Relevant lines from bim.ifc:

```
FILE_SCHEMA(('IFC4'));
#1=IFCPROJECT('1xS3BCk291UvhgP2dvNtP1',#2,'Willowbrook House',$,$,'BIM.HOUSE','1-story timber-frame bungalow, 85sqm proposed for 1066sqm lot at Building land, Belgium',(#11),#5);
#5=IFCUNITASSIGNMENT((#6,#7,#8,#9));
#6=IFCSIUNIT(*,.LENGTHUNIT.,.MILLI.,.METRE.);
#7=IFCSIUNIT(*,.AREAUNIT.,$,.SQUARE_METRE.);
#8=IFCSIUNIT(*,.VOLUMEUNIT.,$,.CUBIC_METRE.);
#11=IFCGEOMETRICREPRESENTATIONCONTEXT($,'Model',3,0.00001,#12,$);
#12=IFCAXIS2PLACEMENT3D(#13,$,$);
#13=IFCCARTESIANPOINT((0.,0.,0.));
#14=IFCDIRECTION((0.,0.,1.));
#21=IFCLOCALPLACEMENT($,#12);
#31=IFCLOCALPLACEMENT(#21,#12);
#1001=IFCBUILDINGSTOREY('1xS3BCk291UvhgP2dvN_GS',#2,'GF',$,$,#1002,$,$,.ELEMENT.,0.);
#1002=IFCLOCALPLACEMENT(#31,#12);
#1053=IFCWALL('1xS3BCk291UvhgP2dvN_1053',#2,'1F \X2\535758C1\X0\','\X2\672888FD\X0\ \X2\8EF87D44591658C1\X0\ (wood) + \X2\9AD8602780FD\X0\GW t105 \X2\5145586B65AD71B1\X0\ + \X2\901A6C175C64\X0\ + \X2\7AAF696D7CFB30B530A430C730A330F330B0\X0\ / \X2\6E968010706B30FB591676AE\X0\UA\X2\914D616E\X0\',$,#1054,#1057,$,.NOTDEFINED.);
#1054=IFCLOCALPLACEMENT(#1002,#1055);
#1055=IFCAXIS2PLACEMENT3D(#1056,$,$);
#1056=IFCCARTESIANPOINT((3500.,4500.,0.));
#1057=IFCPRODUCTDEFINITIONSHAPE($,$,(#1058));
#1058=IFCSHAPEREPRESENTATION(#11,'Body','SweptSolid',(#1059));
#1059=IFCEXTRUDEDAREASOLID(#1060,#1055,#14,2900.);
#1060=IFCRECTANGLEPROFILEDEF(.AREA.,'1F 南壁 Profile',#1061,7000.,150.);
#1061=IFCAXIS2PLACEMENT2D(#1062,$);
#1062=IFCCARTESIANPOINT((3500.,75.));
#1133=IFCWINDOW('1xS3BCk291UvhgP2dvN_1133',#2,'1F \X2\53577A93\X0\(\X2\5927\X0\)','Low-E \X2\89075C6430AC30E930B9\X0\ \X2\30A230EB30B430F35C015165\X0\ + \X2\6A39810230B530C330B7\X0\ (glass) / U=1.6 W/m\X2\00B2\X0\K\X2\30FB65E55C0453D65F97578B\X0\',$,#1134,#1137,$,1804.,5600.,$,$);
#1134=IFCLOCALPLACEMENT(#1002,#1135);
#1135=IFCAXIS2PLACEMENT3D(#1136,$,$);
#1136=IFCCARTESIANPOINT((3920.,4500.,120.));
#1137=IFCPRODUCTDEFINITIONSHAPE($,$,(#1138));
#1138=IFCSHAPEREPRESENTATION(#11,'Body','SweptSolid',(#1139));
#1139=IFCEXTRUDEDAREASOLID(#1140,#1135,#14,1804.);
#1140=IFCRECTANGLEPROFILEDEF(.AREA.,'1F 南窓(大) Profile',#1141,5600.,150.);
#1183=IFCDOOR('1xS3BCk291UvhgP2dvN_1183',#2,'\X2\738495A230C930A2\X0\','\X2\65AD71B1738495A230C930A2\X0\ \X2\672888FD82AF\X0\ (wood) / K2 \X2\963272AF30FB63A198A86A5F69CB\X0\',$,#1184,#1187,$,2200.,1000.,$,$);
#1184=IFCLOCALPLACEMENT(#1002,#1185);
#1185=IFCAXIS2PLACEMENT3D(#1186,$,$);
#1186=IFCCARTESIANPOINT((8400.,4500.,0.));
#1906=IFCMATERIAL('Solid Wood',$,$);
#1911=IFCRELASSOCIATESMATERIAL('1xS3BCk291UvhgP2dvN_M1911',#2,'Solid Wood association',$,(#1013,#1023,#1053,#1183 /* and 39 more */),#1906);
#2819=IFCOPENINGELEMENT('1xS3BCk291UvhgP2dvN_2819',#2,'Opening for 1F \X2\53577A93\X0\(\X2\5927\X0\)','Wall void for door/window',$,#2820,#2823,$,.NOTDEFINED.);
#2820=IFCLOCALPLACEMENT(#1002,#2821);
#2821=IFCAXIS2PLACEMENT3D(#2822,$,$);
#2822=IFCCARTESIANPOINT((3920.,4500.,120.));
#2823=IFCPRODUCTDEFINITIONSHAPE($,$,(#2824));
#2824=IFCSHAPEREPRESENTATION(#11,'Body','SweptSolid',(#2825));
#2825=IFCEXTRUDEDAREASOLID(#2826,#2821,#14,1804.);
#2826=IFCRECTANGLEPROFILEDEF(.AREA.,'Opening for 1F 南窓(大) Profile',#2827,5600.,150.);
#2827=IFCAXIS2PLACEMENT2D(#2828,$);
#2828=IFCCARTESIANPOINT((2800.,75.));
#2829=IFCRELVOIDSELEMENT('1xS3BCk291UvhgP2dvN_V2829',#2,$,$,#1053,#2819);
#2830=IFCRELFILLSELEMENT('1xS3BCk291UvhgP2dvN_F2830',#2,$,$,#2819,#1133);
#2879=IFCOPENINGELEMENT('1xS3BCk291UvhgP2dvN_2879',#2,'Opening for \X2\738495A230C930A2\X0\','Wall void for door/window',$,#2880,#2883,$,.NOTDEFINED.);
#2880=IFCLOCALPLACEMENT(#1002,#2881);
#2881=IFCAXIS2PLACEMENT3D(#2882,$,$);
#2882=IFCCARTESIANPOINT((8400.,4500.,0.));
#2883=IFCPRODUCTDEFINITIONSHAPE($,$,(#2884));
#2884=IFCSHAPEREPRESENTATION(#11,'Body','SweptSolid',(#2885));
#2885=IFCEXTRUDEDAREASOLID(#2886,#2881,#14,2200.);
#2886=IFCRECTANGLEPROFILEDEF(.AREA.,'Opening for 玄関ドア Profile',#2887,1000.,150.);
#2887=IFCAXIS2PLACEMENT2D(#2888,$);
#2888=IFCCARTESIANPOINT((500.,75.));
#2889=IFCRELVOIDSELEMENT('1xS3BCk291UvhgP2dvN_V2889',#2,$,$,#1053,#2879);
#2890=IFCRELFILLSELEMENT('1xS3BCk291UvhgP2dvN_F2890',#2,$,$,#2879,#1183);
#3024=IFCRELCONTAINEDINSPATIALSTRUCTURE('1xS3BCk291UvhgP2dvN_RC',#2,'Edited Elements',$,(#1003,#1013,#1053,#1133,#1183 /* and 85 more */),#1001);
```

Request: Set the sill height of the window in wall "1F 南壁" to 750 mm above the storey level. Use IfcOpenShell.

```python
import numpy as np
import ifcopenshell
import ifcopenshell.api.geometry
import ifcopenshell.geom
import ifcopenshell.util.element
import ifcopenshell.util.placement
import ifcopenshell.util.shape
import ifcopenshell.util.unit

model = ifcopenshell.open("bim.ifc")
unit_scale = ifcopenshell.util.unit.calculate_unit_scale(model)

window = model.by_guid("1xS3BCk291UvhgP2dvN_1133")
opening = window.FillsVoids[0].RelatingOpeningElement
storey = ifcopenshell.util.element.get_container(window, ifc_class="IfcBuildingStorey")
level = ifcopenshell.util.placement.get_local_placement(storey.ObjectPlacement)[2, 3]

# The opening's origin need not be at the sill, so measure its lowest point.
shape = ifcopenshell.geom.create_shape(ifcopenshell.geom.settings(), opening)
bottom = ifcopenshell.util.shape.get_shape_bottom_elevation(shape, shape.geometry) / unit_scale
dz = level + 750.0 - bottom

shift = np.array([0.0, 0.0, dz])
# The window is not placed relative to its opening, so move both.
for product in (opening, window):
    matrix = ifcopenshell.util.placement.get_local_placement(product.ObjectPlacement)
    matrix[:3, 3] += shift
    ifcopenshell.api.geometry.edit_object_placement(model, product=product, matrix=matrix, is_si=False)

print(f"moved by {dz * unit_scale:+.3f} m")

model.write("bim_edited.ifc")
```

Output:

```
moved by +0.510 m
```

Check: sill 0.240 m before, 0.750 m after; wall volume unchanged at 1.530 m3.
